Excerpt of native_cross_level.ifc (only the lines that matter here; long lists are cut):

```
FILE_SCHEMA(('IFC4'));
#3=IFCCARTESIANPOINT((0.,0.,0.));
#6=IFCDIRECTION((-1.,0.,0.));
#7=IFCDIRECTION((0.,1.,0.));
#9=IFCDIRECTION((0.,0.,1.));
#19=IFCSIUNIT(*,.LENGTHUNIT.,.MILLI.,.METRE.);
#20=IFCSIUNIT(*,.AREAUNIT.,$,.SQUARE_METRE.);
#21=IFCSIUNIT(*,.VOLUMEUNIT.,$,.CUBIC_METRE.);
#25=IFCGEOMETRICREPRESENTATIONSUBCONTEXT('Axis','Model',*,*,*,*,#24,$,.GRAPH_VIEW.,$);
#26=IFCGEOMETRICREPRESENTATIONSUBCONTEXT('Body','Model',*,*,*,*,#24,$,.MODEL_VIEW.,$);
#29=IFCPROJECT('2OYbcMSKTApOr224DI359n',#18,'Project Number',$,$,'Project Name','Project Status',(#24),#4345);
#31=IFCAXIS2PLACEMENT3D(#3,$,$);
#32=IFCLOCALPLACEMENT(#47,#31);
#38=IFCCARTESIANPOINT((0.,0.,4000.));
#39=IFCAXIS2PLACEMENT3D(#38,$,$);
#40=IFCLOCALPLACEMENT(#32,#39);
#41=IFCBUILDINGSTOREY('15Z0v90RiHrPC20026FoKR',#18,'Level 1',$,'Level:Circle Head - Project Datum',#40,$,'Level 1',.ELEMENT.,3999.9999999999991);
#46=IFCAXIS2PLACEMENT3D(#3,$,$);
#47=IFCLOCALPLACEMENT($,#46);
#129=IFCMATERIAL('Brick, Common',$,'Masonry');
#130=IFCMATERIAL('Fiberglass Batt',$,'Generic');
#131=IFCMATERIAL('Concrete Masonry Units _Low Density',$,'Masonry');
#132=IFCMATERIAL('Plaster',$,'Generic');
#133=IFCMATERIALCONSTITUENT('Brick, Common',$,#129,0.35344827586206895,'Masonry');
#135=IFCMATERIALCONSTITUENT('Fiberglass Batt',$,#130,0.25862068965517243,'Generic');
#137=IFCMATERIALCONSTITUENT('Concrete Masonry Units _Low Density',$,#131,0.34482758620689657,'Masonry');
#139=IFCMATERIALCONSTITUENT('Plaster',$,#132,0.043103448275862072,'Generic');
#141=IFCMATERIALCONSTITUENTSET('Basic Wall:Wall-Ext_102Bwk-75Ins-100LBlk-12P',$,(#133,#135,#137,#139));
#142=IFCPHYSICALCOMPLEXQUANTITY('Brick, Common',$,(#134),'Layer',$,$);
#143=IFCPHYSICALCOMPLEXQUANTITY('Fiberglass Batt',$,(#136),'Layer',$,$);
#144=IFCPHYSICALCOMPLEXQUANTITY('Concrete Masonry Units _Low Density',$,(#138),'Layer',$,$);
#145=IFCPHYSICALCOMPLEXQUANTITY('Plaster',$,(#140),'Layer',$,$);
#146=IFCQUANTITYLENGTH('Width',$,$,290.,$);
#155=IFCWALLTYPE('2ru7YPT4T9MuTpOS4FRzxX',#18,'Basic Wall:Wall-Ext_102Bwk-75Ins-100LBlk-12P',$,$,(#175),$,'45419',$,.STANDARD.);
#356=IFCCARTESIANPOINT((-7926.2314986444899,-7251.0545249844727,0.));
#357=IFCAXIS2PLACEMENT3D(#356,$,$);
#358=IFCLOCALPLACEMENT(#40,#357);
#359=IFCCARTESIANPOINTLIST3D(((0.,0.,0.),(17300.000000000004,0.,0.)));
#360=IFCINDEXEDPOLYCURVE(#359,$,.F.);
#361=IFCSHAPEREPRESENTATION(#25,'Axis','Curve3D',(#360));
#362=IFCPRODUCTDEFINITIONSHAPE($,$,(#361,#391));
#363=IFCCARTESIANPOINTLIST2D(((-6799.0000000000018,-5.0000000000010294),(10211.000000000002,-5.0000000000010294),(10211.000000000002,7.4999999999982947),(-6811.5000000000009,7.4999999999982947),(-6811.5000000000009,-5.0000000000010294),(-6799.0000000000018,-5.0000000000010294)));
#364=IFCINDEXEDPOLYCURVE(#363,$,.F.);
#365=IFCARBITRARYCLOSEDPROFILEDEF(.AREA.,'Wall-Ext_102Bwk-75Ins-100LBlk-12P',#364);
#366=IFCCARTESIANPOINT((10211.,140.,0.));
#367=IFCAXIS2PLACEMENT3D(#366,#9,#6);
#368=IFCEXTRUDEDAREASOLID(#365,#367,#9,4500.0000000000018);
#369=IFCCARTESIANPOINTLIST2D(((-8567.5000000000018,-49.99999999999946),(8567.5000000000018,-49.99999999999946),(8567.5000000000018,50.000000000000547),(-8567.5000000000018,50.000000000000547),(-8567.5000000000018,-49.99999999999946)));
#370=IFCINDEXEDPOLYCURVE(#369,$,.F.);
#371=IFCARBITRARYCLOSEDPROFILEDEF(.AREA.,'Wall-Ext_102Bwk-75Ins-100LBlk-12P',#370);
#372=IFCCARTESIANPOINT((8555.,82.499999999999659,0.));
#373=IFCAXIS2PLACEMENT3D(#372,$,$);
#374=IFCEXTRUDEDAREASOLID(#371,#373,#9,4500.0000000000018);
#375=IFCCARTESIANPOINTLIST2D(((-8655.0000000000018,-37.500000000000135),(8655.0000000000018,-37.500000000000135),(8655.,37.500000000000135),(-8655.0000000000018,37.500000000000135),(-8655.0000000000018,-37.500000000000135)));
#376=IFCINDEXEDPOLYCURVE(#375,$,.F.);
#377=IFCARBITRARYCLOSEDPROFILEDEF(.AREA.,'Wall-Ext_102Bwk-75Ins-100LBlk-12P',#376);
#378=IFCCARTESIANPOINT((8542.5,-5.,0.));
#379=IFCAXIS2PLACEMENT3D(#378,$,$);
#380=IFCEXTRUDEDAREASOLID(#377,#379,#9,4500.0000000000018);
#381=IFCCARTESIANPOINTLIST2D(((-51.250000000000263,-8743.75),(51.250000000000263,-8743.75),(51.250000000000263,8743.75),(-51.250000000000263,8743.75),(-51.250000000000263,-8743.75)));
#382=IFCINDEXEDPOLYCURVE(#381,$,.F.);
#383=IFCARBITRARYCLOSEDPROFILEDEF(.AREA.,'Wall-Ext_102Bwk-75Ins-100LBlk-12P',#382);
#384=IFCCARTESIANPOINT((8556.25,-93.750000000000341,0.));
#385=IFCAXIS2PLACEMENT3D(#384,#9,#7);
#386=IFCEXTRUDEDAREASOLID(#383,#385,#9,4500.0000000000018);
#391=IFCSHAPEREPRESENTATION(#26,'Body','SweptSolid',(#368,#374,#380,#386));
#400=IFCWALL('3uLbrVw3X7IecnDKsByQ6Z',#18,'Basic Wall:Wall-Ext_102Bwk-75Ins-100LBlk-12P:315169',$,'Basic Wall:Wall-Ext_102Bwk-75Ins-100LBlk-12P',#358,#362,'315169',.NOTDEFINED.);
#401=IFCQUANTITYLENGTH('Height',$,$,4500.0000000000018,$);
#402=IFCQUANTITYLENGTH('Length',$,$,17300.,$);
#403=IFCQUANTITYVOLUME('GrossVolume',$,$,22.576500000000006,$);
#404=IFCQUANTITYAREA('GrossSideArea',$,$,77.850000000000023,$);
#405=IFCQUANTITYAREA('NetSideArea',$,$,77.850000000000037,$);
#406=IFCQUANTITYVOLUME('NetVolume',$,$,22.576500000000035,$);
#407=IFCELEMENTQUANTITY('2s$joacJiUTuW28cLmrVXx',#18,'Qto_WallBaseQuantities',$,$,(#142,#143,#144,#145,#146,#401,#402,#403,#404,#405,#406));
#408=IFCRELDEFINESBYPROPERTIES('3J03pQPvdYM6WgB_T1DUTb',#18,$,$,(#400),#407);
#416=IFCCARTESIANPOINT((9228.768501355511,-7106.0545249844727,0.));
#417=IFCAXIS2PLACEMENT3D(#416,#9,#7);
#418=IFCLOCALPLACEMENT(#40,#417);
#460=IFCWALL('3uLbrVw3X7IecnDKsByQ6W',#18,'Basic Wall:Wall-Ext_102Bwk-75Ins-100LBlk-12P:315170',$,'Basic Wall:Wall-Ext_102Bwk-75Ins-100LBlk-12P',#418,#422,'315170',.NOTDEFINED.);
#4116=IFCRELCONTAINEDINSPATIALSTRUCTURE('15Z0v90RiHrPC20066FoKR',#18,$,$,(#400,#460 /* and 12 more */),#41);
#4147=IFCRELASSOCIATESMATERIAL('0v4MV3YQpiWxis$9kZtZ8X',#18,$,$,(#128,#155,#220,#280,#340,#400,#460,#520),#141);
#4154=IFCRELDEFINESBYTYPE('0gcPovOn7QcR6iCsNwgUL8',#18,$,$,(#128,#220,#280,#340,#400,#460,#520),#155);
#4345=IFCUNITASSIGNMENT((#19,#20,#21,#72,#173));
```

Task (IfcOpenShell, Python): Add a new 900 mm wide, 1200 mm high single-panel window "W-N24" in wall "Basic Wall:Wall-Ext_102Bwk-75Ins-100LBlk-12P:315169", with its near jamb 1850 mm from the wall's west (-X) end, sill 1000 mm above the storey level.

```python
import numpy as np
import ifcopenshell
import ifcopenshell.api.feature
import ifcopenshell.api.geometry
import ifcopenshell.api.pset
import ifcopenshell.api.root
import ifcopenshell.api.spatial
import ifcopenshell.geom
import ifcopenshell.util.element
import ifcopenshell.util.placement
import ifcopenshell.util.representation
import ifcopenshell.util.shape
import ifcopenshell.util.unit

model = ifcopenshell.open("native_cross_level.ifc")
unit_scale = ifcopenshell.util.unit.calculate_unit_scale(model)
area_scale = ifcopenshell.util.unit.calculate_unit_scale(model, "AREAUNIT")
volume_scale = ifcopenshell.util.unit.calculate_unit_scale(model, "VOLUMEUNIT")
settings = ifcopenshell.geom.settings()


def volume(element):
    """Net volume in cubic metres, openings subtracted."""
    shape = ifcopenshell.geom.create_shape(settings, element)
    return ifcopenshell.util.shape.get_volume(shape.geometry)


wall = model.by_id(400)
storey = ifcopenshell.util.element.get_container(wall, ifc_class="IfcBuildingStorey")
context = ifcopenshell.util.representation.get_context(model, "Model", "Body", "MODEL_VIEW")
before = volume(wall)

width, height, from_end, sill = 0.9, 1.2, 1.85, 1  # metres

# The wall runs along its own X axis, and the end named is its -X end.
wall_shape = ifcopenshell.geom.create_shape(settings, wall)
x, y, z = ifcopenshell.util.shape.get_vertices(wall_shape.geometry).T
start = x.min() + from_end
face, thickness = float(y.min()), float(y.max() - y.min())
wall_matrix = ifcopenshell.util.placement.get_local_placement(wall.ObjectPlacement)
level = ifcopenshell.util.placement.get_local_placement(storey.ObjectPlacement)[2, 3]


def in_wall(x, y):
    """Placement at x, y metres in the wall's axes, at sill height."""
    matrix = wall_matrix.copy()
    matrix[:, 3] = wall_matrix @ np.array([x / unit_scale, y / unit_scale, 0.0, 1.0])
    matrix[2, 3] = level + sill / unit_scale
    return matrix


# Opening: a box that overshoots both wall faces by 50 mm.
opening = ifcopenshell.api.root.create_entity(model, ifc_class="IfcOpeningElement", predefined_type="OPENING")
box = ifcopenshell.api.geometry.add_wall_representation(
    model, context=context, length=width, height=height, thickness=thickness + 0.1
)
ifcopenshell.api.geometry.assign_representation(model, product=opening, representation=box)
ifcopenshell.api.geometry.edit_object_placement(model, product=opening, matrix=in_wall(start, face - 0.05), is_si=False)
ifcopenshell.api.feature.add_feature(model, feature=opening, element=wall)

window = ifcopenshell.api.root.create_entity(model, ifc_class="IfcWindow", name="W-N24", predefined_type="WINDOW")
window.OverallWidth, window.OverallHeight = width / unit_scale, height / unit_scale
window.PartitioningType = "SINGLE_PANEL"
body = ifcopenshell.api.geometry.add_window_representation(
    model,
    context=context,
    overall_width=window.OverallWidth,
    overall_height=window.OverallHeight,
    partition_type="SINGLE_PANEL",
)
ifcopenshell.api.geometry.assign_representation(model, product=window, representation=body)
ifcopenshell.api.spatial.assign_container(model, products=[window], relating_structure=storey)
ifcopenshell.api.feature.add_filling(model, opening=opening, element=window)

# Centre the window in the wall's thickness.
ifcopenshell.api.geometry.edit_object_placement(model, product=window, matrix=in_wall(start, face), is_si=False)
window_shape = ifcopenshell.geom.create_shape(settings, window)
depth = ifcopenshell.util.shape.get_vertices(window_shape.geometry)[:, 1]
offset = face + thickness / 2 - (depth.min() + depth.max()) / 2
ifcopenshell.api.geometry.edit_object_placement(model, product=window, matrix=in_wall(start, offset), is_si=False)

after = volume(wall)

# Update the wall's stored quantities.
qto = model.by_id(ifcopenshell.util.element.get_pset(wall, "Qto_WallBaseQuantities", should_inherit=False)["id"])
ifcopenshell.api.pset.edit_qto(model, qto=qto, properties={
    "NetSideArea": after / thickness / area_scale,
    "NetVolume": after / volume_scale,
})

print(f"wall volume {before:.3f} -> {after:.3f} m3")

model.write("native_cross_level_updated.ifc")
```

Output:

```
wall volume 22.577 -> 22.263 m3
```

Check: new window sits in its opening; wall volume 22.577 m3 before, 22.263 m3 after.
